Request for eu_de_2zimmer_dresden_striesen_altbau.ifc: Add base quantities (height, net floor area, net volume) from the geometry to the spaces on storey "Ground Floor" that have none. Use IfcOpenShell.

First a look at what the model holds.

```python
import ifcopenshell
import ifcopenshell.util.element
import ifcopenshell.util.unit

model = ifcopenshell.open("eu_de_2zimmer_dresden_striesen_altbau.ifc")
print(model.schema)
for unit_type in ("LENGTHUNIT", "AREAUNIT", "VOLUMEUNIT"):
    print(unit_type, ifcopenshell.util.unit.calculate_unit_scale(model, unit_type))
storey = next(s for s in model.by_type("IfcBuildingStorey") if s.Name == "Ground Floor")
spaces = [e for e in ifcopenshell.util.element.get_decomposition(storey) if e.is_a("IfcSpace")]
for e in sorted(spaces, key=lambda e: e.id()):
    print(e.id(), e.is_a(), e.Name, list(ifcopenshell.util.element.get_psets(e, qtos_only=True)), sep=" | ")
```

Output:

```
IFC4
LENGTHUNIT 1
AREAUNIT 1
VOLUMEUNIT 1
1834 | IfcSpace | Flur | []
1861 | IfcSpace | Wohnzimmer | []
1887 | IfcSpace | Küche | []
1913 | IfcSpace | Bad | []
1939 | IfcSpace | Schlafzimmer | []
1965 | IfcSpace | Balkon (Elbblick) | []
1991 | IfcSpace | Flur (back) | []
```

```python
import ifcopenshell
import ifcopenshell.api.pset
import ifcopenshell.geom
import ifcopenshell.util.element
import ifcopenshell.util.shape
import ifcopenshell.util.unit

model = ifcopenshell.open("eu_de_2zimmer_dresden_striesen_altbau.ifc")
unit_scale = ifcopenshell.util.unit.calculate_unit_scale(model)
area_scale = ifcopenshell.util.unit.calculate_unit_scale(model, "AREAUNIT")
volume_scale = ifcopenshell.util.unit.calculate_unit_scale(model, "VOLUMEUNIT")
settings = ifcopenshell.geom.settings()

storey = next(s for s in model.by_type("IfcBuildingStorey") if s.Name == "Ground Floor")
spaces = [e for e in ifcopenshell.util.element.get_decomposition(storey) if e.is_a("IfcSpace")]

for e in sorted(spaces, key=lambda e: e.id()):
    if ifcopenshell.util.element.get_psets(e, qtos_only=True, should_inherit=False):
        continue
    # Geometry comes back in metres, in the element's own axes.
    shape = ifcopenshell.geom.create_shape(settings, e)
    values = {
        "Height": ifcopenshell.util.shape.get_z(shape.geometry) / unit_scale,
        "NetFloorArea": ifcopenshell.util.shape.get_footprint_area(shape.geometry) / area_scale,
        "NetVolume": ifcopenshell.util.shape.get_volume(shape.geometry) / volume_scale,
    }
    qto = ifcopenshell.api.pset.add_qto(model, product=e, name="Qto_SpaceBaseQuantities")
    ifcopenshell.api.pset.edit_qto(model, qto=qto, properties=values)
    print(e.id(), {k: round(v, 3) for k, v in values.items()})

model.write("eu_de_2zimmer_dresden_striesen_altbau_updated.ifc")
```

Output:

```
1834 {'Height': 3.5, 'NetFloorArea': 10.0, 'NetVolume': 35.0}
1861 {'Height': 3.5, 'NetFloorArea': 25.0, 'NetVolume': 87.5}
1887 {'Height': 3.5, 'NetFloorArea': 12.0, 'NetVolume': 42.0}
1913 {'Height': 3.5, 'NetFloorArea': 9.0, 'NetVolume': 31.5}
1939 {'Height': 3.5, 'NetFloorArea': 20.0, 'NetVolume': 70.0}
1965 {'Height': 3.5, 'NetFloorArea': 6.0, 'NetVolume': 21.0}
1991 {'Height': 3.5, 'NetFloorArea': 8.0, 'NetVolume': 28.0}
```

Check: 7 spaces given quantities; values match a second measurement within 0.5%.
